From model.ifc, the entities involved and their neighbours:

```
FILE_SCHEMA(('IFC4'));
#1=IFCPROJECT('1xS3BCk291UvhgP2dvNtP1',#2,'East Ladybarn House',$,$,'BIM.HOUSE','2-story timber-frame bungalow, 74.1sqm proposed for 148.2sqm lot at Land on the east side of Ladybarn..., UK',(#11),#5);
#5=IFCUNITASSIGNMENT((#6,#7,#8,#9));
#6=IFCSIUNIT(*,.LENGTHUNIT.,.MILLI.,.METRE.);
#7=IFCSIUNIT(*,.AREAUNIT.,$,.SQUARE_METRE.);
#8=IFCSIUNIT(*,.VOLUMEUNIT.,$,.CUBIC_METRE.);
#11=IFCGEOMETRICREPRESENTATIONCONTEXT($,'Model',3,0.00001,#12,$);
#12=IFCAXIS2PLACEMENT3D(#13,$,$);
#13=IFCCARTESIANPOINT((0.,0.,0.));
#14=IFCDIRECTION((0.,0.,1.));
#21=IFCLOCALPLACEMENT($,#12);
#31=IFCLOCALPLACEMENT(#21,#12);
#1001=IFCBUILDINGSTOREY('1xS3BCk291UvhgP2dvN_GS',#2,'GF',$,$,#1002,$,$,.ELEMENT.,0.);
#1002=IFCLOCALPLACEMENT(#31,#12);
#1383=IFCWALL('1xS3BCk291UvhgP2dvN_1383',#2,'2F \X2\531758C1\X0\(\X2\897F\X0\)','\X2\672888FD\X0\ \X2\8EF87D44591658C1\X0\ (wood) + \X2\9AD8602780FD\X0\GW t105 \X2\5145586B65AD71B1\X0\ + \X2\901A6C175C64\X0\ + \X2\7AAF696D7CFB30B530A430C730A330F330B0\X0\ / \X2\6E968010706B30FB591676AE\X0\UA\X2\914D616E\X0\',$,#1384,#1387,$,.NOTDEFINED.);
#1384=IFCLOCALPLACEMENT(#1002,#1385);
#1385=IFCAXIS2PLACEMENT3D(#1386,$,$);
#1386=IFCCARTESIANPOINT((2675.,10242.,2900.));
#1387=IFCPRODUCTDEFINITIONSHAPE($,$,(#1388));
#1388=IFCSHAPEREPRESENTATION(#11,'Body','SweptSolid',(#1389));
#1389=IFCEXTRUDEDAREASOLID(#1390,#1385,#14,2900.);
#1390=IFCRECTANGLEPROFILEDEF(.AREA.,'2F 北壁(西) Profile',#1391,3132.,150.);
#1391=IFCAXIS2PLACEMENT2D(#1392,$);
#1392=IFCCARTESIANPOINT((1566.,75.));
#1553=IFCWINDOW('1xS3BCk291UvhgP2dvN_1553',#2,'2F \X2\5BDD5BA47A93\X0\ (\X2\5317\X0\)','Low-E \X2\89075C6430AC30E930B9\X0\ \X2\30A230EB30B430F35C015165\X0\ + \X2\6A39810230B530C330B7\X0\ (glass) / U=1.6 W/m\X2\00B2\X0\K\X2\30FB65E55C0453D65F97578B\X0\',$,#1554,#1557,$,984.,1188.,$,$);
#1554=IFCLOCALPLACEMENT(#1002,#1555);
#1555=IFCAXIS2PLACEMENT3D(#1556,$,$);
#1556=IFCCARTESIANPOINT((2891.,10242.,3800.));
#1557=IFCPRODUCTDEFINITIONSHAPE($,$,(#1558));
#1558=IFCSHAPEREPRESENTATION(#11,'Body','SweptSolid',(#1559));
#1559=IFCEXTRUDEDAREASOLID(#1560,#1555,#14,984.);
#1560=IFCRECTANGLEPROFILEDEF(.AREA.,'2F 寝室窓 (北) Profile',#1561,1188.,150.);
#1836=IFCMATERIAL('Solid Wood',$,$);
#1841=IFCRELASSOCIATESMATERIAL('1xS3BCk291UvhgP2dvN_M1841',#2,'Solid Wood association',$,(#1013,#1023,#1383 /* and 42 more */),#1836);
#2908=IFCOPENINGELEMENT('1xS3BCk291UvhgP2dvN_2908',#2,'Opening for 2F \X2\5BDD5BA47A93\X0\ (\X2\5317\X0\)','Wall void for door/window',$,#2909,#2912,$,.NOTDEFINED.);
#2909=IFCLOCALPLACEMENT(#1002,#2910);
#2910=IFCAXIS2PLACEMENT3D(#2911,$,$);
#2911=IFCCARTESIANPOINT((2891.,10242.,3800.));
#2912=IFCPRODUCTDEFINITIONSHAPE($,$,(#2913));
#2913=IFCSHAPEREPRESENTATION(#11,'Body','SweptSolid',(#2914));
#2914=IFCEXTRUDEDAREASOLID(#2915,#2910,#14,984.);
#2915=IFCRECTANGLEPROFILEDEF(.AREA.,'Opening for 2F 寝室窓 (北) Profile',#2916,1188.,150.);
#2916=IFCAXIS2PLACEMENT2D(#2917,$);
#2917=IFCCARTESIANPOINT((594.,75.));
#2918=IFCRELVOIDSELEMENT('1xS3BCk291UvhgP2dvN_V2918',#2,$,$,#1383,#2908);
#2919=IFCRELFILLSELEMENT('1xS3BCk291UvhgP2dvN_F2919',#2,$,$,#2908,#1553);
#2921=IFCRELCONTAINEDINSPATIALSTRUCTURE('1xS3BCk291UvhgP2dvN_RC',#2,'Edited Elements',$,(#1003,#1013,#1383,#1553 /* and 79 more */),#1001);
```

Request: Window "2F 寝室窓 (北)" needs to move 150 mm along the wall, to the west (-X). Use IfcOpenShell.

```python
import ifcopenshell
import ifcopenshell.api.geometry
import ifcopenshell.util.placement
import ifcopenshell.util.unit

model = ifcopenshell.open("model.ifc")
unit_scale = ifcopenshell.util.unit.calculate_unit_scale(model)

window = model.by_id(1553)
opening = window.FillsVoids[0].RelatingOpeningElement
wall = opening.VoidsElements[0].RelatingBuildingElement

wall_matrix = ifcopenshell.util.placement.get_local_placement(wall.ObjectPlacement)
shift = wall_matrix[:3, 0] * -0.15 / unit_scale
before = ifcopenshell.util.placement.get_local_placement(window.ObjectPlacement)[:3, 3].copy()

# The window is not placed relative to its opening, so move both.
for product in (opening, window):
    matrix = ifcopenshell.util.placement.get_local_placement(product.ObjectPlacement)
    matrix[:3, 3] += shift
    ifcopenshell.api.geometry.edit_object_placement(model, product=product, matrix=matrix, is_si=False)

after = ifcopenshell.util.placement.get_local_placement(window.ObjectPlacement)[:3, 3]
print("window moved by", (after - before).round(3) + 0.0)

model.write("model-out.ifc")
```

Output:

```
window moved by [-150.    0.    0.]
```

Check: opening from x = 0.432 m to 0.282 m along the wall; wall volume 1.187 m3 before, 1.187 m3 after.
